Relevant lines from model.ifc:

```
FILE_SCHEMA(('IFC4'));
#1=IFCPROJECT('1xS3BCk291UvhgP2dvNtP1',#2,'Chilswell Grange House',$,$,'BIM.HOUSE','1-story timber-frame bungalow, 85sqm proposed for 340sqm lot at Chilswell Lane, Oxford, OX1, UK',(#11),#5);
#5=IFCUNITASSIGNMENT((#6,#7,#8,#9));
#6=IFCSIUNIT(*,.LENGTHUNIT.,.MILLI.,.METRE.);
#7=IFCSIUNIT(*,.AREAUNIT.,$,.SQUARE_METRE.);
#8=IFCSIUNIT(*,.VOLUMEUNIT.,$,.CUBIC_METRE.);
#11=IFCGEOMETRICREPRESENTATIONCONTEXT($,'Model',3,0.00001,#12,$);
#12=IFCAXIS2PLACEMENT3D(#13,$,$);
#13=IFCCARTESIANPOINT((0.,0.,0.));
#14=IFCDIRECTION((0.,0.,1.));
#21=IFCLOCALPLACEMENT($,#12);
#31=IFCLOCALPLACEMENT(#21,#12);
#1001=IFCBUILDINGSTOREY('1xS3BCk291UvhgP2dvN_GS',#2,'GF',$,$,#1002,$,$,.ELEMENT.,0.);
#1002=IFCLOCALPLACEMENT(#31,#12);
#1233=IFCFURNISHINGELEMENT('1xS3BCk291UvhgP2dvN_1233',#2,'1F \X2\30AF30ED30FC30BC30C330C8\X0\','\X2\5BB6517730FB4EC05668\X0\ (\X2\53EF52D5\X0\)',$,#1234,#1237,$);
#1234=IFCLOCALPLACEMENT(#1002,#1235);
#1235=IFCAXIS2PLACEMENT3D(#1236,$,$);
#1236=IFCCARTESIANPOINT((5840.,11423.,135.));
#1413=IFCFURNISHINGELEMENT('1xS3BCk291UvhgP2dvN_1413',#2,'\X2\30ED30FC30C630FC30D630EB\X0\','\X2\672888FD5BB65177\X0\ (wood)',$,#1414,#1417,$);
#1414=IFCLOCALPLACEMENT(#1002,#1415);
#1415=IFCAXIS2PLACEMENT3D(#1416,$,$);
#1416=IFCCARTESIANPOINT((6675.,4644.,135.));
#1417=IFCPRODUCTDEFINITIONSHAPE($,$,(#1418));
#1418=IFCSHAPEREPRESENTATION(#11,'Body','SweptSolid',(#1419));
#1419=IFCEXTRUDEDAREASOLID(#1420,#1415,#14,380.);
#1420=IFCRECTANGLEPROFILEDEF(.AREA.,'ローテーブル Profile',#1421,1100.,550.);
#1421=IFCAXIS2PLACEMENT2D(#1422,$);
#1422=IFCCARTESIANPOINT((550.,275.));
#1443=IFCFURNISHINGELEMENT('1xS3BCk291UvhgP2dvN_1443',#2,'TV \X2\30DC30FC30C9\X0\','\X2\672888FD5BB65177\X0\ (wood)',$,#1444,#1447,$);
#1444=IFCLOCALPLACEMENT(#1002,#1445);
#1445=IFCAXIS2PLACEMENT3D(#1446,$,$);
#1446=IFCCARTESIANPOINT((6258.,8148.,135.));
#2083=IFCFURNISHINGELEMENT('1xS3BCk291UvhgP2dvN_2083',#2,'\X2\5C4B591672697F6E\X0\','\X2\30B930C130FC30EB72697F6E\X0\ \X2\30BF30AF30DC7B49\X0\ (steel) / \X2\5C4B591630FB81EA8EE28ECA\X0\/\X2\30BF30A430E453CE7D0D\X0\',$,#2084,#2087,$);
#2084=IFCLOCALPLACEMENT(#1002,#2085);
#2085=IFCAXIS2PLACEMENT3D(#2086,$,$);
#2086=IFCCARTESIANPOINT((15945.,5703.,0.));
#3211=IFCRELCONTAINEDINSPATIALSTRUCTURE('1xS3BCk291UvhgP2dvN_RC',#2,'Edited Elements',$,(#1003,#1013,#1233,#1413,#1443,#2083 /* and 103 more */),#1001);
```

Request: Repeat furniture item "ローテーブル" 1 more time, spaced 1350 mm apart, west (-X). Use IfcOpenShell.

```python
import numpy as np
import ifcopenshell
import ifcopenshell.api.geometry
import ifcopenshell.api.root
import ifcopenshell.util.element
import ifcopenshell.util.placement

model = ifcopenshell.open("model.ifc")


def reuse_history(source, copy):
    """copy_class also copies each property set's owner history, people and application; keep the originals."""
    for rel in copy.IsDefinedBy:
        if rel.is_a("IfcRelDefinesByProperties") and (history := rel.RelatingPropertyDefinition.OwnerHistory):
            rel.RelatingPropertyDefinition.OwnerHistory = source.OwnerHistory
            ifcopenshell.util.element.remove_deep2(model, history)


source = model.by_guid("1xS3BCk291UvhgP2dvN_1413")
base = ifcopenshell.util.placement.get_local_placement(source.ObjectPlacement)
step = np.array([-1.0, 0.0, 0.0]) * 1350.0

for i in range(1, 2):
    copy = ifcopenshell.api.root.copy_class(model, product=source)
    copy.Representation = ifcopenshell.util.element.copy_deep(
        model, source.Representation, exclude=["IfcGeometricRepresentationContext", "IfcRepresentationMap"]
    )
    reuse_history(source, copy)
    matrix = base.copy()
    matrix[:3, 3] += i * step
    print("added at", matrix[:3, 3].round(3) + 0.0)
    ifcopenshell.api.geometry.edit_object_placement(model, product=copy, matrix=matrix, is_si=False)

model.write("model-out.ifc")
```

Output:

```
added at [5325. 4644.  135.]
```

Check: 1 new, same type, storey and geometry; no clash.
